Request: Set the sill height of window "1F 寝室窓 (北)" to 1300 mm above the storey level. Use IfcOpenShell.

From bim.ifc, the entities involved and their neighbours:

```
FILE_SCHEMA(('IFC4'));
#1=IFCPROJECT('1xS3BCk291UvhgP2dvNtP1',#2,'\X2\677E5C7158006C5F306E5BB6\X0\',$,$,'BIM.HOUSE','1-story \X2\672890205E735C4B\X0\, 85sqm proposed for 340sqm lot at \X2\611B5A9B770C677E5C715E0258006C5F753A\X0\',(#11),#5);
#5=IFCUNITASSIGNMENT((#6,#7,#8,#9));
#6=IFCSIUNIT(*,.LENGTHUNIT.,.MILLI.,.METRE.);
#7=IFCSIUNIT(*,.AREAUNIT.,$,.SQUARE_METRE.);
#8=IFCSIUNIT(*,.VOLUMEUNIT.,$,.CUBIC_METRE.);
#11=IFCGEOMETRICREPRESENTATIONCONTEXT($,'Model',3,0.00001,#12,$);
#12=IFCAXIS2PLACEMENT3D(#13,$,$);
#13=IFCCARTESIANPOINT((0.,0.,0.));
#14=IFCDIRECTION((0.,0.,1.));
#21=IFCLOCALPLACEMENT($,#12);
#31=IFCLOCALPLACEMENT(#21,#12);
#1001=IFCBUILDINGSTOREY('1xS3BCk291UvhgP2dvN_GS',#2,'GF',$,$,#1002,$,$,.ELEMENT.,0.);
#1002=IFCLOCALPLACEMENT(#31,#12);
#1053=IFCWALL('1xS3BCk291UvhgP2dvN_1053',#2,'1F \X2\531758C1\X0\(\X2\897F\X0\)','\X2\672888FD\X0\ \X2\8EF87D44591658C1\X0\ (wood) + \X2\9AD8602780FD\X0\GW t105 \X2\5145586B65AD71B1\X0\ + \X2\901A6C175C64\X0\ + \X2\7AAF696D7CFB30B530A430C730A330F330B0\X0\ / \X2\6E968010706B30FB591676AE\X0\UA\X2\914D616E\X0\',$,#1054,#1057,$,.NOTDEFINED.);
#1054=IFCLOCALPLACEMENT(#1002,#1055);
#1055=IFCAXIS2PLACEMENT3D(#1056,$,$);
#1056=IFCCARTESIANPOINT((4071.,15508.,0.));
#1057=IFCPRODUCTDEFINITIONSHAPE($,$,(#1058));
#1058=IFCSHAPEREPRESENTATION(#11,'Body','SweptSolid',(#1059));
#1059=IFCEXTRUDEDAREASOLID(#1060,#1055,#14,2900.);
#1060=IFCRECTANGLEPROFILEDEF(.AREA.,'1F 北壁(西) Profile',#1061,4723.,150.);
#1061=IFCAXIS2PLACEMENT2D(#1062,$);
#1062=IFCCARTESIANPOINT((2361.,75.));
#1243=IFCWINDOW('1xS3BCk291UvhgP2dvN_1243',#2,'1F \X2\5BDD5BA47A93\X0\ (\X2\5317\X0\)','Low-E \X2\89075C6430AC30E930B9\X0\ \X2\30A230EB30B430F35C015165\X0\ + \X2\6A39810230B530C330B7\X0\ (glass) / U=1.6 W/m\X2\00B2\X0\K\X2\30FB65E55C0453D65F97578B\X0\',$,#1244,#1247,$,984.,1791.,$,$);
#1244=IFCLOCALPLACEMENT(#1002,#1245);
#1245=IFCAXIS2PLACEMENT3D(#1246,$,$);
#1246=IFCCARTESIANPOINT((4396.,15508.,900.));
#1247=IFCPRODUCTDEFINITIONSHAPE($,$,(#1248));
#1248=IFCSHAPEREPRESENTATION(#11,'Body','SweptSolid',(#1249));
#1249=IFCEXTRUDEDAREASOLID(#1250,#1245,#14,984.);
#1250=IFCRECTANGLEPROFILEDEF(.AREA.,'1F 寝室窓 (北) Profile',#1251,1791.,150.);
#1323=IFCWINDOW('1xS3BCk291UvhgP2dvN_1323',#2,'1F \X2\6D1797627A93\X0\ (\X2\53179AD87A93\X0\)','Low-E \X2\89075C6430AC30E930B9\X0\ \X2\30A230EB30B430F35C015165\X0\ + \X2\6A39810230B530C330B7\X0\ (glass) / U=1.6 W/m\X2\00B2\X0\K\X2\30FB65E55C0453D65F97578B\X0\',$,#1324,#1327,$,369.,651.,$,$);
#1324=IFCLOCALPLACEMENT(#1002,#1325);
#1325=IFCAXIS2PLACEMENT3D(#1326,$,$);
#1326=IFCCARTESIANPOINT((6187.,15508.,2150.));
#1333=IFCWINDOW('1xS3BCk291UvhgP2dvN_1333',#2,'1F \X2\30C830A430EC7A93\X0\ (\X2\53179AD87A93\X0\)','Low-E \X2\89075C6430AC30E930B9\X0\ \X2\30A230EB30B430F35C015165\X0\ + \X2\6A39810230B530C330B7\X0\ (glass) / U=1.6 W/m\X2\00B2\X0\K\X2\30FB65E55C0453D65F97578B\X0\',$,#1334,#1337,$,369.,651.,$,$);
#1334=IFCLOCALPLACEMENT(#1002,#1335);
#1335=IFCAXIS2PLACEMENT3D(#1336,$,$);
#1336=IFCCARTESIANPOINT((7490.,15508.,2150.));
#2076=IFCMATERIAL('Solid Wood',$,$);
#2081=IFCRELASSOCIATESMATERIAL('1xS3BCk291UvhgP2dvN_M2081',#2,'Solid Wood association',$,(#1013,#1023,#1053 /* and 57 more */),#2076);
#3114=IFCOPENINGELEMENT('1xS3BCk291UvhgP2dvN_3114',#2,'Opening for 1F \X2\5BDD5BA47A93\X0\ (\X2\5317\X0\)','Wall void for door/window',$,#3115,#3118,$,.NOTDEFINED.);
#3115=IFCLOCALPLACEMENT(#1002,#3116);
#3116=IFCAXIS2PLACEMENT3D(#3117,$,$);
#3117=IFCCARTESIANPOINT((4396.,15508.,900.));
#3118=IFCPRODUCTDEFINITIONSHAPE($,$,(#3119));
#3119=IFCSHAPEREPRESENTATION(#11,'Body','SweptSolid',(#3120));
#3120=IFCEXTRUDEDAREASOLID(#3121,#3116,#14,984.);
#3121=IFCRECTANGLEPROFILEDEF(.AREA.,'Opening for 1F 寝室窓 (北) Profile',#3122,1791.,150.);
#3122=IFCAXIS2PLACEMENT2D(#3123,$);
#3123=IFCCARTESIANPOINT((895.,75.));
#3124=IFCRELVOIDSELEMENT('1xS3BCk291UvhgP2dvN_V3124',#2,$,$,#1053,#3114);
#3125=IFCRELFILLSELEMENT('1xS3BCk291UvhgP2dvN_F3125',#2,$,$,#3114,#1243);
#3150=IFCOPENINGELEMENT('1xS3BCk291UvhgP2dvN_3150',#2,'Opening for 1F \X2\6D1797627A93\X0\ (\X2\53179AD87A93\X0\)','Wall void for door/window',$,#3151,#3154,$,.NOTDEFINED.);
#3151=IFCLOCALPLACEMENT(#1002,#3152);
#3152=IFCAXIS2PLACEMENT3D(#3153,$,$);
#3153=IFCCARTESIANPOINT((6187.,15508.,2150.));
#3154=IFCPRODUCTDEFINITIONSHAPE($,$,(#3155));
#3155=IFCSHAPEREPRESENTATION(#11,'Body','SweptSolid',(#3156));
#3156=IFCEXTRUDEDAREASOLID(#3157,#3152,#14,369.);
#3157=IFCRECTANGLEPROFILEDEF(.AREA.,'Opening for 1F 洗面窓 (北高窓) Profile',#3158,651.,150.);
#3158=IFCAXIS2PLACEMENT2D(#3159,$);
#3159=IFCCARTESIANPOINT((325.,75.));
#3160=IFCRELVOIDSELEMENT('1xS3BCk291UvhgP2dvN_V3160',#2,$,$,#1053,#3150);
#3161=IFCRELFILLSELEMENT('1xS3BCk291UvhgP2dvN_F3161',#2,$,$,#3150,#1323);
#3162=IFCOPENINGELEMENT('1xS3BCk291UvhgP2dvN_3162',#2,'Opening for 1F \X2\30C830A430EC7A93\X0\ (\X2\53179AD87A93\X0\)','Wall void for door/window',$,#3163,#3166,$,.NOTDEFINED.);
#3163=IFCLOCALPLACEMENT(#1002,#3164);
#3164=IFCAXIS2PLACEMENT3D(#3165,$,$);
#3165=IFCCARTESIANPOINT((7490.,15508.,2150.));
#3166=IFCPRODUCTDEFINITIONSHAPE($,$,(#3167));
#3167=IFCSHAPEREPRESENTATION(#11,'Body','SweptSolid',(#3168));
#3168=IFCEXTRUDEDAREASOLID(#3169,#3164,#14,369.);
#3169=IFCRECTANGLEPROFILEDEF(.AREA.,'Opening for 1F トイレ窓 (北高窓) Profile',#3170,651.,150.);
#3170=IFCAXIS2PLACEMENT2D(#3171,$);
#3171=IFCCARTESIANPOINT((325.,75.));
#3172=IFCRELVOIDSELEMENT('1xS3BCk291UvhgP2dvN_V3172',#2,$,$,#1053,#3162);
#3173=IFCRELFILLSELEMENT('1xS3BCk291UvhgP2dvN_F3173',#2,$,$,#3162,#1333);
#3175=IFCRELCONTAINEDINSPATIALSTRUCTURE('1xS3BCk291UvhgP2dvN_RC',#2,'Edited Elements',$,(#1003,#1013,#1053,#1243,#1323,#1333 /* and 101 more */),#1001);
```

```python
import numpy as np
import ifcopenshell
import ifcopenshell.api.geometry
import ifcopenshell.geom
import ifcopenshell.util.element
import ifcopenshell.util.placement
import ifcopenshell.util.shape
import ifcopenshell.util.unit

model = ifcopenshell.open("bim.ifc")
unit_scale = ifcopenshell.util.unit.calculate_unit_scale(model)

window = model.by_guid("1xS3BCk291UvhgP2dvN_1243")
opening = window.FillsVoids[0].RelatingOpeningElement
storey = ifcopenshell.util.element.get_container(window, ifc_class="IfcBuildingStorey")
level = ifcopenshell.util.placement.get_local_placement(storey.ObjectPlacement)[2, 3]

# The opening's origin need not be at the sill, so measure its lowest point.
shape = ifcopenshell.geom.create_shape(ifcopenshell.geom.settings(), opening)
bottom = ifcopenshell.util.shape.get_shape_bottom_elevation(shape, shape.geometry) / unit_scale
dz = level + 1.3 / unit_scale - bottom

shift = np.array([0.0, 0.0, dz])
# The window is not placed relative to its opening, so move both.
for product in (opening, window):
    matrix = ifcopenshell.util.placement.get_local_placement(product.ObjectPlacement)
    matrix[:3, 3] += shift
    ifcopenshell.api.geometry.edit_object_placement(model, product=product, matrix=matrix, is_si=False)

print(f"moved by {dz * unit_scale:+.3f} m")

model.write("bim-out.ifc")
```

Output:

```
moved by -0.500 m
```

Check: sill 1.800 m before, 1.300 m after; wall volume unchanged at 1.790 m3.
